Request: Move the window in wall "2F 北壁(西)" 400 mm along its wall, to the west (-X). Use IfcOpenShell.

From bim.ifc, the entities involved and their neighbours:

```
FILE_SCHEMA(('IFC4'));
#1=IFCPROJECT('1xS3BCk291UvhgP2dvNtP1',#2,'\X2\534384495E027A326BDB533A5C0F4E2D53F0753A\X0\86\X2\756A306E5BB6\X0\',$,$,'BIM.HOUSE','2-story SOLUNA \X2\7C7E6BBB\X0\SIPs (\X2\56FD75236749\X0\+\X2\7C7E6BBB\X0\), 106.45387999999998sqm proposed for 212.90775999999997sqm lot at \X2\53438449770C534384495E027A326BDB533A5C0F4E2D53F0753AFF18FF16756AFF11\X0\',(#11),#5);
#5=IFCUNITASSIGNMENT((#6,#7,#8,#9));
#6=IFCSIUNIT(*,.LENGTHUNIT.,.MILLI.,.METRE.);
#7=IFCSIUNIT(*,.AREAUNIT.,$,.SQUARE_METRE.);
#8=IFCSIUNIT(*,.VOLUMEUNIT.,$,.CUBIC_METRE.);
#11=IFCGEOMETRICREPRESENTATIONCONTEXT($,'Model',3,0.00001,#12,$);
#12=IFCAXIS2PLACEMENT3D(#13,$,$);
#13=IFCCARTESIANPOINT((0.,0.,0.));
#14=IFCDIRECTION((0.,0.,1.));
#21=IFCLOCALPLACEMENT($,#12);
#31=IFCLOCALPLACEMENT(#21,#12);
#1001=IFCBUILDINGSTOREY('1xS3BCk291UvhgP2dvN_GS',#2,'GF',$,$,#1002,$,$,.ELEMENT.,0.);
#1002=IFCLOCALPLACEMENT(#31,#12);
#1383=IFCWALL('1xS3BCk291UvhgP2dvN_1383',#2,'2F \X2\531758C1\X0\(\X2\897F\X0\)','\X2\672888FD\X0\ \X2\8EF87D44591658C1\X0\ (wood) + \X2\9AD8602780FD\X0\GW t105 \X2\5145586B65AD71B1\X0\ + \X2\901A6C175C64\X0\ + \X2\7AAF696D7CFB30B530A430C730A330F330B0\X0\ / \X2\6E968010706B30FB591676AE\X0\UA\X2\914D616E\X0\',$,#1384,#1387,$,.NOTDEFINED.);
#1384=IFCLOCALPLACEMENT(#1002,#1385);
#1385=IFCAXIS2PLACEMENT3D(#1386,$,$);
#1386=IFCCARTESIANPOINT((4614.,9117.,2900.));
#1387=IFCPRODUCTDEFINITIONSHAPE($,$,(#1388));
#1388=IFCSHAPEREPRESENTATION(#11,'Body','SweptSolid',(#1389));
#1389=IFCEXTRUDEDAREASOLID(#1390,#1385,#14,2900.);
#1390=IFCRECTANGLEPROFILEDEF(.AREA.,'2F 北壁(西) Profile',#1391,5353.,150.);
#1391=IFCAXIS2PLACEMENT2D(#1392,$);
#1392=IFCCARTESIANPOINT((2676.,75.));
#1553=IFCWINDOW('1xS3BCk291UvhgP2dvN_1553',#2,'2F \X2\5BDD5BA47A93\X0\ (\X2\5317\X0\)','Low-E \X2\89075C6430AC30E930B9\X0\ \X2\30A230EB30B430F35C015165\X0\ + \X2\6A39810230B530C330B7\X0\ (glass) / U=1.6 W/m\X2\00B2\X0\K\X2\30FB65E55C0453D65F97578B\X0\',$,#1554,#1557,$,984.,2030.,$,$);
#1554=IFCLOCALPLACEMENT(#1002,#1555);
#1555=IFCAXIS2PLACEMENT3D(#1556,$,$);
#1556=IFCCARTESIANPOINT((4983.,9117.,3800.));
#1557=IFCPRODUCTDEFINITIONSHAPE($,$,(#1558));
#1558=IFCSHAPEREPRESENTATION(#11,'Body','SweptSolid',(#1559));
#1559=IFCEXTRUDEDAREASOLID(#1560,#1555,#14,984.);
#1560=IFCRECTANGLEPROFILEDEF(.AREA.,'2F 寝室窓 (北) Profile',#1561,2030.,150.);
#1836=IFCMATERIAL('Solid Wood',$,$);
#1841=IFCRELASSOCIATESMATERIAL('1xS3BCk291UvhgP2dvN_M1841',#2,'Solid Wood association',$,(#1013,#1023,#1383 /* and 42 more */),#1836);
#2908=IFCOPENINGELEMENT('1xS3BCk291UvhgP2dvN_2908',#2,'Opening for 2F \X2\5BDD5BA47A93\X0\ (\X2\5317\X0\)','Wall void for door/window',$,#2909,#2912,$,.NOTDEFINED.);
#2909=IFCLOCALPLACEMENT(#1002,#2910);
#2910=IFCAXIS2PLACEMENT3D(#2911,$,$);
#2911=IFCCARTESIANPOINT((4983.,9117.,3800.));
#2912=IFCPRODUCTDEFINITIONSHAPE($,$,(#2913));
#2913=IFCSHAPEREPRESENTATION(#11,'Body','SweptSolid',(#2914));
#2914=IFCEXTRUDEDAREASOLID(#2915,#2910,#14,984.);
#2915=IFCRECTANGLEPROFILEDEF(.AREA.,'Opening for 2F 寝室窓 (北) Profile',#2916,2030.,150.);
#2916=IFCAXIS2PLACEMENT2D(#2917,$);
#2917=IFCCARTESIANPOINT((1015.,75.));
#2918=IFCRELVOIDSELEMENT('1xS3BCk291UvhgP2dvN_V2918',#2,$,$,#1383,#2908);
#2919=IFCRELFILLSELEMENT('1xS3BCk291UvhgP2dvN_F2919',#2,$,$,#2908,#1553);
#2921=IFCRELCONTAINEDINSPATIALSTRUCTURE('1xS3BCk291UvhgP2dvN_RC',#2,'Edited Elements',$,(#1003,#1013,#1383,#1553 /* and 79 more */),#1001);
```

```python
import ifcopenshell
import ifcopenshell.api.geometry
import ifcopenshell.util.placement
import ifcopenshell.util.unit

model = ifcopenshell.open("bim.ifc")
unit_scale = ifcopenshell.util.unit.calculate_unit_scale(model)

window = model.by_guid("1xS3BCk291UvhgP2dvN_1553")
opening = window.FillsVoids[0].RelatingOpeningElement
wall = opening.VoidsElements[0].RelatingBuildingElement

wall_matrix = ifcopenshell.util.placement.get_local_placement(wall.ObjectPlacement)
shift = wall_matrix[:3, 0] * -0.4 / unit_scale
before = ifcopenshell.util.placement.get_local_placement(window.ObjectPlacement)[:3, 3].copy()

# The window is not placed relative to its opening, so move both.
for product in (opening, window):
    matrix = ifcopenshell.util.placement.get_local_placement(product.ObjectPlacement)
    matrix[:3, 3] += shift
    ifcopenshell.api.geometry.edit_object_placement(model, product=product, matrix=matrix, is_si=False)

after = ifcopenshell.util.placement.get_local_placement(window.ObjectPlacement)[:3, 3]
print("window moved by", (after - before).round(3) + 0.0)

model.write("bim_rev.ifc")
```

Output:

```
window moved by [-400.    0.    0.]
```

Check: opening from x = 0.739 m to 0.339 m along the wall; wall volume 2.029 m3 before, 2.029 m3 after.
